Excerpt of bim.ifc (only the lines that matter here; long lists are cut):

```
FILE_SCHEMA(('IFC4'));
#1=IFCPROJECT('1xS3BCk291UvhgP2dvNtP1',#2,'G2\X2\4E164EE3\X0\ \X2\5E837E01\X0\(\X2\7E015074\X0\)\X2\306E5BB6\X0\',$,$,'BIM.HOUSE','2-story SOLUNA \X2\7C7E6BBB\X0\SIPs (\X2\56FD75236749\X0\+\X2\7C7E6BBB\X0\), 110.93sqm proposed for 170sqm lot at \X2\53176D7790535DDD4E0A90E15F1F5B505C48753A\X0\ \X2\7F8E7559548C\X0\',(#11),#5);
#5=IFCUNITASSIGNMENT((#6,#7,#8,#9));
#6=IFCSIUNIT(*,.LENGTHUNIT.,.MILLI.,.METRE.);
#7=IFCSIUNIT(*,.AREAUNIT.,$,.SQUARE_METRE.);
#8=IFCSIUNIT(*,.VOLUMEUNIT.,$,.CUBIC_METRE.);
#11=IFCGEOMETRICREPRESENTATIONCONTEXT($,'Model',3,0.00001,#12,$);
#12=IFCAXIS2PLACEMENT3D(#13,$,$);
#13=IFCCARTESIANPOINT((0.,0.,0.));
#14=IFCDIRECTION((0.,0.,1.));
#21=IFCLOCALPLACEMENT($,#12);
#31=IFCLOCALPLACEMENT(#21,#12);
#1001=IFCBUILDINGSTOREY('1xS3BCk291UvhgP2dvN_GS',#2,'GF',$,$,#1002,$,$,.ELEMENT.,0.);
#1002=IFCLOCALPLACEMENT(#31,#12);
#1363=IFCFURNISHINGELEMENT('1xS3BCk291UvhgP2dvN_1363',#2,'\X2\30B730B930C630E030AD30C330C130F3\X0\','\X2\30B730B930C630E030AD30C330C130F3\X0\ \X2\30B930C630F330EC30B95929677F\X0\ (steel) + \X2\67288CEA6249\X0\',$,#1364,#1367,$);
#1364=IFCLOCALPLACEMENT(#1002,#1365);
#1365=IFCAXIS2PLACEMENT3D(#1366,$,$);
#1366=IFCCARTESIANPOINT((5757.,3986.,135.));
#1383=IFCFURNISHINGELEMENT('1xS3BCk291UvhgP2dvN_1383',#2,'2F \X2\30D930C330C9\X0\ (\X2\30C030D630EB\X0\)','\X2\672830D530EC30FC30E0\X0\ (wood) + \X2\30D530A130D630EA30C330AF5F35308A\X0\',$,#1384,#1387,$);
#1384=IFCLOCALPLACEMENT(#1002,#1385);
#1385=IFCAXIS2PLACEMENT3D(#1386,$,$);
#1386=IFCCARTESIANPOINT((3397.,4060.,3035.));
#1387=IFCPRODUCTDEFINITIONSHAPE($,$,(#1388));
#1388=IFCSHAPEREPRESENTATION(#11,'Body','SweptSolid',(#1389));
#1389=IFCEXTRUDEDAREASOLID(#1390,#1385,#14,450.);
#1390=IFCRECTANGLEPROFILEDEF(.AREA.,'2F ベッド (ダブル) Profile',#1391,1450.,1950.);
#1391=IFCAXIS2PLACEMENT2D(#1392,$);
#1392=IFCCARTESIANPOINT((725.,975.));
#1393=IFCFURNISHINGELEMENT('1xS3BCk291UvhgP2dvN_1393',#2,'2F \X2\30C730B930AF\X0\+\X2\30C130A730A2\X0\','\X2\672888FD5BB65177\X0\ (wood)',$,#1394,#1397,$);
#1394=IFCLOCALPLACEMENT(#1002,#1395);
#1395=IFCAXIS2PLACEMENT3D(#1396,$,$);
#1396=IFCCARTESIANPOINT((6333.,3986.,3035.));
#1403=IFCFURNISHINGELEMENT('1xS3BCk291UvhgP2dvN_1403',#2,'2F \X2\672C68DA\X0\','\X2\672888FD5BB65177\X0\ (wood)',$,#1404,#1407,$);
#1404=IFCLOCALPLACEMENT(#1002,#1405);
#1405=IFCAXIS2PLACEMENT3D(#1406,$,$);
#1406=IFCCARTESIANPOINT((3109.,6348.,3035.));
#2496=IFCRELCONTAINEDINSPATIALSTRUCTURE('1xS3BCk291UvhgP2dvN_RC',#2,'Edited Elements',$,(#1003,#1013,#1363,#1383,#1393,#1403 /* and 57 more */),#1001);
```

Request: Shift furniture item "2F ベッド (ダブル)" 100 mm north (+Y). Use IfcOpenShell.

```python
import ifcopenshell
import ifcopenshell.api.geometry
import ifcopenshell.util.placement
import ifcopenshell.util.unit

model = ifcopenshell.open("bim.ifc")
unit_scale = ifcopenshell.util.unit.calculate_unit_scale(model)

item = model.by_guid("1xS3BCk291UvhgP2dvN_1383")
matrix = ifcopenshell.util.placement.get_local_placement(item.ObjectPlacement)
matrix[1, 3] += 0.1 / unit_scale
ifcopenshell.api.geometry.edit_object_placement(model, product=item, matrix=matrix, is_si=False)

print(ifcopenshell.util.placement.get_local_placement(item.ObjectPlacement).round(3) + 0.0)

model.write("bim_v2.ifc")
```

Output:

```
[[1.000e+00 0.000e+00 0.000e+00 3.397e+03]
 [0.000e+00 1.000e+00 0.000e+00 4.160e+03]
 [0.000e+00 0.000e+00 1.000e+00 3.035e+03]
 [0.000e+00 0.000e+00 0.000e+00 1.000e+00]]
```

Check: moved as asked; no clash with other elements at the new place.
